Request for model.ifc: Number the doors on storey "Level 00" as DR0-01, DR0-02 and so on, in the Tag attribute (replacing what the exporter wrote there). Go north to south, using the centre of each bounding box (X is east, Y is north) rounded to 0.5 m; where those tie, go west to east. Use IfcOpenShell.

First a look at what the model holds.

```python
import ifcopenshell
import ifcopenshell.util.element
import ifcopenshell.util.placement

model = ifcopenshell.open("model.ifc")
print(model.schema)
storey = next(s for s in model.by_type("IfcBuildingStorey") if s.Name == "Level 00")
doors = [e for e in ifcopenshell.util.element.get_decomposition(storey) if e.is_a("IfcDoor")]
for e in sorted(doors, key=lambda e: e.id()):
    origin = ifcopenshell.util.placement.get_local_placement(e.ObjectPlacement)[:3, 3]
    print(e.id(), e.Tag, e.Name, origin.round(2) + 0.0, sep=" | ")
```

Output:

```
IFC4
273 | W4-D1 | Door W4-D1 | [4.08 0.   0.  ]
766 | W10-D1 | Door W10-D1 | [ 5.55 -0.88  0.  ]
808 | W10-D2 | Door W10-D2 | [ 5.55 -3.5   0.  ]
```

```python
import ifcopenshell
import ifcopenshell.geom
import ifcopenshell.util.element
import ifcopenshell.util.shape

model = ifcopenshell.open("model.ifc")
settings = ifcopenshell.geom.settings()
settings.set("use-world-coords", True)


def centre(element):
    shape = ifcopenshell.geom.create_shape(settings, element)
    return ifcopenshell.util.shape.get_bbox_centroid(shape.geometry)


storey = next(s for s in model.by_type("IfcBuildingStorey") if s.Name == "Level 00")
doors = [e for e in ifcopenshell.util.element.get_decomposition(storey) if e.is_a("IfcDoor")]

# Insertion points can sit at a corner or the storey origin, so sort by the geometry (in metres).
centres = {e: centre(e) for e in doors}
doors.sort(key=lambda e: (-round(centres[e][1] / 0.5), centres[e][0]))

for i, e in enumerate(doors, start=1):
    number = f"DR0-{i:02d}"
    e.Tag = number
    print(e.id(), number)

model.write("model_v2.ifc")
```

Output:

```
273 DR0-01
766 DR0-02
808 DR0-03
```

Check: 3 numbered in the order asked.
